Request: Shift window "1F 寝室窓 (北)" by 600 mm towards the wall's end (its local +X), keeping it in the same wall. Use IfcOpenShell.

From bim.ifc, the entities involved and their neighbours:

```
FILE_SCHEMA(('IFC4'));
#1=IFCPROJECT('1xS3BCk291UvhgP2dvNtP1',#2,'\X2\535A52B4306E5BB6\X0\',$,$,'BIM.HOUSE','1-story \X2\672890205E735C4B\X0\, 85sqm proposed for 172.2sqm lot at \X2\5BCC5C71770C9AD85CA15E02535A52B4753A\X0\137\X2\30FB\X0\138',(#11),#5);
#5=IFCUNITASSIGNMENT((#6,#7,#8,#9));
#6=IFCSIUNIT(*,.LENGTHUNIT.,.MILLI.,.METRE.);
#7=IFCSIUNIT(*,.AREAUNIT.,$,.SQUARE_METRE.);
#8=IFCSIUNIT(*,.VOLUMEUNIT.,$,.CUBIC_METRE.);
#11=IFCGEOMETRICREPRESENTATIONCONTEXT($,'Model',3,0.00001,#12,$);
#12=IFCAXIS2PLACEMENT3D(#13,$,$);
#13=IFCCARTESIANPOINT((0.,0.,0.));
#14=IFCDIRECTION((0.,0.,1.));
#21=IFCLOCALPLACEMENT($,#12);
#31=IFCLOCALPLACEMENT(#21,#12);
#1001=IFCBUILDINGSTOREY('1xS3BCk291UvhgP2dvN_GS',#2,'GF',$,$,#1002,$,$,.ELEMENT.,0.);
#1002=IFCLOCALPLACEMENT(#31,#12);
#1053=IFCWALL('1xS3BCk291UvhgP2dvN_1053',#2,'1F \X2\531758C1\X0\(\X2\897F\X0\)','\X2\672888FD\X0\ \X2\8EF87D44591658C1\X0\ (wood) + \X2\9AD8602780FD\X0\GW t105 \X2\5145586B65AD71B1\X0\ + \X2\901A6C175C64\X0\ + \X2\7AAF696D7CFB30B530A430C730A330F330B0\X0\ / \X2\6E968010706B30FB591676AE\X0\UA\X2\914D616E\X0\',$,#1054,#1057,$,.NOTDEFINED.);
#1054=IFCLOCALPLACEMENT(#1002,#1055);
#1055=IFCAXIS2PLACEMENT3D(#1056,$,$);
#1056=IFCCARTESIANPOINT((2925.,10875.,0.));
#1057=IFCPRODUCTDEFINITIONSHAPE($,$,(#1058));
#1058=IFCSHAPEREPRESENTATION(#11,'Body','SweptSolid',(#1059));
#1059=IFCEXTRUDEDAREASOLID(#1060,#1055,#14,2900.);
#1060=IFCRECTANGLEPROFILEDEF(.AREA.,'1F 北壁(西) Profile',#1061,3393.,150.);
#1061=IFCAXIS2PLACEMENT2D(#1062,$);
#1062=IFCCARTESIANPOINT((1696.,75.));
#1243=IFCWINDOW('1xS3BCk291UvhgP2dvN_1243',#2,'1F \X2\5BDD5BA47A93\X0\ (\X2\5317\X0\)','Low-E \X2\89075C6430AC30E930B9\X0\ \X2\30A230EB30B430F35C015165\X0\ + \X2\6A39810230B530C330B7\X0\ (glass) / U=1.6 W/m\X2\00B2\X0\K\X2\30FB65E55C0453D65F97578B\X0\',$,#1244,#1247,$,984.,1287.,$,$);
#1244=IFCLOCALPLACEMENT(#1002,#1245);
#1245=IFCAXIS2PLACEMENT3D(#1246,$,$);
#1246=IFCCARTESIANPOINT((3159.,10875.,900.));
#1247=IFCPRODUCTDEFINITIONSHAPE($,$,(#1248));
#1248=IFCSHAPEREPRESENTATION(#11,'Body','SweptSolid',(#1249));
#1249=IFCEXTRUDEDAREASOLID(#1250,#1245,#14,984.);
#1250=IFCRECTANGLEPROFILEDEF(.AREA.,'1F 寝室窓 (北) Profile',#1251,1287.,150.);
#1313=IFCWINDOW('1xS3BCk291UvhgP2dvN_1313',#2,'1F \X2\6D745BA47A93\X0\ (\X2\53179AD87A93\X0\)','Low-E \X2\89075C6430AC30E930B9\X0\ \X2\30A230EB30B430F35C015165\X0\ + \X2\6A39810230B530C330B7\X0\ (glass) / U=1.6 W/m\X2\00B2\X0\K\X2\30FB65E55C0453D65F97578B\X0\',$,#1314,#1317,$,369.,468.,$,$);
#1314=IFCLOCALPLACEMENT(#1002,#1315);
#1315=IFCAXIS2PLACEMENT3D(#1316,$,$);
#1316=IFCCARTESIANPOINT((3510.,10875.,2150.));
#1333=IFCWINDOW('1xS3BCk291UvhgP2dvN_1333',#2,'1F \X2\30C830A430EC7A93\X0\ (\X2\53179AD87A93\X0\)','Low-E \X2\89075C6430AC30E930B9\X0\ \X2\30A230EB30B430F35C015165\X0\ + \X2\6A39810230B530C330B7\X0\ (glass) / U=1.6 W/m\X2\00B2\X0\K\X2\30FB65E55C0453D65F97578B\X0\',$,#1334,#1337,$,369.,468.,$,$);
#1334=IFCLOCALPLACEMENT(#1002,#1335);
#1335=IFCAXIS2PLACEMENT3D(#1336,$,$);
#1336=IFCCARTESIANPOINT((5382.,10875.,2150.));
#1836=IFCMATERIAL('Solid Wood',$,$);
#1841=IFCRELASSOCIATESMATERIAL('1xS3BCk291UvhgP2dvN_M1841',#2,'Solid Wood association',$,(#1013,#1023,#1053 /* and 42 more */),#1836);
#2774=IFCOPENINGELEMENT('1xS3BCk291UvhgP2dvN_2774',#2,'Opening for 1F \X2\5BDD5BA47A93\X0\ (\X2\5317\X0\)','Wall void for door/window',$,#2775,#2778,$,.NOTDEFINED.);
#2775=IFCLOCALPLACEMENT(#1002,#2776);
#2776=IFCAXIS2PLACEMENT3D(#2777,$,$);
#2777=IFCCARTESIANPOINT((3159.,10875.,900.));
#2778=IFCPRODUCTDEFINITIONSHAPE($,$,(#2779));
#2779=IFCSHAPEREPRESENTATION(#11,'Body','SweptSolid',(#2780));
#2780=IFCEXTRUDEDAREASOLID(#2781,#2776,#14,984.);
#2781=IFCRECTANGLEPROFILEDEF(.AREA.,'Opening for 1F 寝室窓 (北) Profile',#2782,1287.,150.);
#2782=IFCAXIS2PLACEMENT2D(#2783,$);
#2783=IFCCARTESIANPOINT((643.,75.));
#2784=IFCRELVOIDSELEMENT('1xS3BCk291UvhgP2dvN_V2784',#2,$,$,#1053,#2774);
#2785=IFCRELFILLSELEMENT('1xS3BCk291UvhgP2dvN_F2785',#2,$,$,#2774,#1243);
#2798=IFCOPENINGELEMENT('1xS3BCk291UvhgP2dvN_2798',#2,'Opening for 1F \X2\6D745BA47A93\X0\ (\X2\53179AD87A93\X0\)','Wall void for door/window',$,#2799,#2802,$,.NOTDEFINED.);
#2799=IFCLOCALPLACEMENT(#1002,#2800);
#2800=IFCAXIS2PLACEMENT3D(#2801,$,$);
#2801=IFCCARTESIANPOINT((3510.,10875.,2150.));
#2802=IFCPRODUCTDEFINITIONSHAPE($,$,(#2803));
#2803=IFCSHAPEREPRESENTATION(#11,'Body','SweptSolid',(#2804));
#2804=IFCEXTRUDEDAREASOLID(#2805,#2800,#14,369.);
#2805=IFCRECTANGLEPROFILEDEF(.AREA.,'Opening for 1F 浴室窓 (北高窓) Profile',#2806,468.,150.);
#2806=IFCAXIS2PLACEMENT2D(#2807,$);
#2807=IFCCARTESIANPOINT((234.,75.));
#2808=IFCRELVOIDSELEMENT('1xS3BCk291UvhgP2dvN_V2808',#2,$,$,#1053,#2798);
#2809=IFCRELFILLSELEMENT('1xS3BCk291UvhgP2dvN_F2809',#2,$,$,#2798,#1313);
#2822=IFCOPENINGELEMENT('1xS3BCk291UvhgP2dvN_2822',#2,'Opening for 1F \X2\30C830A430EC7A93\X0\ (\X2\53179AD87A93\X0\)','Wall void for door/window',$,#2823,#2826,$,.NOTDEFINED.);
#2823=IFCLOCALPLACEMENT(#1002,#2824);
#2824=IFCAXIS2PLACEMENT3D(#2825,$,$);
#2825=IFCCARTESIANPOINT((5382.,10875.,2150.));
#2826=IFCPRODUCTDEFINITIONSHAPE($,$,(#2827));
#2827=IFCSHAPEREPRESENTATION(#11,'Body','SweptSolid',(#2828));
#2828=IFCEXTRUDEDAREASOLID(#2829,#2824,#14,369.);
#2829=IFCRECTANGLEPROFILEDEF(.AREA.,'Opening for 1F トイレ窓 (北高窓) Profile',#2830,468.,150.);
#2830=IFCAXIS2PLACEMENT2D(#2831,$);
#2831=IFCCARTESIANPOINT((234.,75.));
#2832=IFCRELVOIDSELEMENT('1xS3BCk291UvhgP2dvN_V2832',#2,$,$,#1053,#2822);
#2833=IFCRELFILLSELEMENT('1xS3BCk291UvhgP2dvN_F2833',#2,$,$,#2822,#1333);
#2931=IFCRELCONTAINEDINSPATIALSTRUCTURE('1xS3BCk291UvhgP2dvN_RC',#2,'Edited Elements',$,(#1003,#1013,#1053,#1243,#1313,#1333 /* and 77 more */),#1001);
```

```python
import ifcopenshell
import ifcopenshell.api.geometry
import ifcopenshell.util.placement

model = ifcopenshell.open("bim.ifc")

window = model.by_id(1243)
opening = window.FillsVoids[0].RelatingOpeningElement
wall = opening.VoidsElements[0].RelatingBuildingElement

wall_matrix = ifcopenshell.util.placement.get_local_placement(wall.ObjectPlacement)
shift = wall_matrix[:3, 0] * 600.0
before = ifcopenshell.util.placement.get_local_placement(window.ObjectPlacement)[:3, 3].copy()

# The window is not placed relative to its opening, so move both.
for product in (opening, window):
    matrix = ifcopenshell.util.placement.get_local_placement(product.ObjectPlacement)
    matrix[:3, 3] += shift
    ifcopenshell.api.geometry.edit_object_placement(model, product=product, matrix=matrix, is_si=False)

after = ifcopenshell.util.placement.get_local_placement(window.ObjectPlacement)[:3, 3]
print("window moved by", (after - before).round(3) + 0.0)

model.write("bim_updated.ifc")
```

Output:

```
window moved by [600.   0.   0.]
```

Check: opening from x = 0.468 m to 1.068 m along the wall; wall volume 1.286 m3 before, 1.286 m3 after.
